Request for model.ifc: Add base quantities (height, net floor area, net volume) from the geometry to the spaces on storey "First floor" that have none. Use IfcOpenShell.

First a look at what the model holds.

```python
import ifcopenshell
import ifcopenshell.util.element
import ifcopenshell.util.unit

model = ifcopenshell.open("model.ifc")
print(model.schema)
for unit_type in ("LENGTHUNIT", "AREAUNIT", "VOLUMEUNIT"):
    print(unit_type, ifcopenshell.util.unit.calculate_unit_scale(model, unit_type))
storey = next(s for s in model.by_type("IfcBuildingStorey") if s.Name == "First floor")
spaces = [e for e in ifcopenshell.util.element.get_decomposition(storey) if e.is_a("IfcSpace")]
for e in sorted(spaces, key=lambda e: e.id()):
    print(e.id(), e.is_a(), e.Name, list(ifcopenshell.util.element.get_psets(e, qtos_only=True)), sep=" | ")
```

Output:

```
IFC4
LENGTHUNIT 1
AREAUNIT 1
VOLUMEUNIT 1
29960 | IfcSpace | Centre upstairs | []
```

```python
import ifcopenshell
import ifcopenshell.api.pset
import ifcopenshell.geom
import ifcopenshell.util.element
import ifcopenshell.util.shape
import ifcopenshell.util.unit

model = ifcopenshell.open("model.ifc")
unit_scale = ifcopenshell.util.unit.calculate_unit_scale(model)
area_scale = ifcopenshell.util.unit.calculate_unit_scale(model, "AREAUNIT")
volume_scale = ifcopenshell.util.unit.calculate_unit_scale(model, "VOLUMEUNIT")
settings = ifcopenshell.geom.settings()

storey = next(s for s in model.by_type("IfcBuildingStorey") if s.Name == "First floor")
spaces = [e for e in ifcopenshell.util.element.get_decomposition(storey) if e.is_a("IfcSpace")]

for e in sorted(spaces, key=lambda e: e.id()):
    if ifcopenshell.util.element.get_psets(e, qtos_only=True, should_inherit=False):
        continue
    # Geometry comes back in metres, in the element's own axes.
    shape = ifcopenshell.geom.create_shape(settings, e)
    values = {
        "Height": ifcopenshell.util.shape.get_z(shape.geometry) / unit_scale,
        "NetFloorArea": ifcopenshell.util.shape.get_footprint_area(shape.geometry) / area_scale,
        "NetVolume": ifcopenshell.util.shape.get_volume(shape.geometry) / volume_scale,
    }
    qto = ifcopenshell.api.pset.add_qto(model, product=e, name="Qto_SpaceBaseQuantities")
    ifcopenshell.api.pset.edit_qto(model, qto=qto, properties=values)
    print(e.id(), {k: round(v, 3) for k, v in values.items()})

model.write("model_updated.ifc")
```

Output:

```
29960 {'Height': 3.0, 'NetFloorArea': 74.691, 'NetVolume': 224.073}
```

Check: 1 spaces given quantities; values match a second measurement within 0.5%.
